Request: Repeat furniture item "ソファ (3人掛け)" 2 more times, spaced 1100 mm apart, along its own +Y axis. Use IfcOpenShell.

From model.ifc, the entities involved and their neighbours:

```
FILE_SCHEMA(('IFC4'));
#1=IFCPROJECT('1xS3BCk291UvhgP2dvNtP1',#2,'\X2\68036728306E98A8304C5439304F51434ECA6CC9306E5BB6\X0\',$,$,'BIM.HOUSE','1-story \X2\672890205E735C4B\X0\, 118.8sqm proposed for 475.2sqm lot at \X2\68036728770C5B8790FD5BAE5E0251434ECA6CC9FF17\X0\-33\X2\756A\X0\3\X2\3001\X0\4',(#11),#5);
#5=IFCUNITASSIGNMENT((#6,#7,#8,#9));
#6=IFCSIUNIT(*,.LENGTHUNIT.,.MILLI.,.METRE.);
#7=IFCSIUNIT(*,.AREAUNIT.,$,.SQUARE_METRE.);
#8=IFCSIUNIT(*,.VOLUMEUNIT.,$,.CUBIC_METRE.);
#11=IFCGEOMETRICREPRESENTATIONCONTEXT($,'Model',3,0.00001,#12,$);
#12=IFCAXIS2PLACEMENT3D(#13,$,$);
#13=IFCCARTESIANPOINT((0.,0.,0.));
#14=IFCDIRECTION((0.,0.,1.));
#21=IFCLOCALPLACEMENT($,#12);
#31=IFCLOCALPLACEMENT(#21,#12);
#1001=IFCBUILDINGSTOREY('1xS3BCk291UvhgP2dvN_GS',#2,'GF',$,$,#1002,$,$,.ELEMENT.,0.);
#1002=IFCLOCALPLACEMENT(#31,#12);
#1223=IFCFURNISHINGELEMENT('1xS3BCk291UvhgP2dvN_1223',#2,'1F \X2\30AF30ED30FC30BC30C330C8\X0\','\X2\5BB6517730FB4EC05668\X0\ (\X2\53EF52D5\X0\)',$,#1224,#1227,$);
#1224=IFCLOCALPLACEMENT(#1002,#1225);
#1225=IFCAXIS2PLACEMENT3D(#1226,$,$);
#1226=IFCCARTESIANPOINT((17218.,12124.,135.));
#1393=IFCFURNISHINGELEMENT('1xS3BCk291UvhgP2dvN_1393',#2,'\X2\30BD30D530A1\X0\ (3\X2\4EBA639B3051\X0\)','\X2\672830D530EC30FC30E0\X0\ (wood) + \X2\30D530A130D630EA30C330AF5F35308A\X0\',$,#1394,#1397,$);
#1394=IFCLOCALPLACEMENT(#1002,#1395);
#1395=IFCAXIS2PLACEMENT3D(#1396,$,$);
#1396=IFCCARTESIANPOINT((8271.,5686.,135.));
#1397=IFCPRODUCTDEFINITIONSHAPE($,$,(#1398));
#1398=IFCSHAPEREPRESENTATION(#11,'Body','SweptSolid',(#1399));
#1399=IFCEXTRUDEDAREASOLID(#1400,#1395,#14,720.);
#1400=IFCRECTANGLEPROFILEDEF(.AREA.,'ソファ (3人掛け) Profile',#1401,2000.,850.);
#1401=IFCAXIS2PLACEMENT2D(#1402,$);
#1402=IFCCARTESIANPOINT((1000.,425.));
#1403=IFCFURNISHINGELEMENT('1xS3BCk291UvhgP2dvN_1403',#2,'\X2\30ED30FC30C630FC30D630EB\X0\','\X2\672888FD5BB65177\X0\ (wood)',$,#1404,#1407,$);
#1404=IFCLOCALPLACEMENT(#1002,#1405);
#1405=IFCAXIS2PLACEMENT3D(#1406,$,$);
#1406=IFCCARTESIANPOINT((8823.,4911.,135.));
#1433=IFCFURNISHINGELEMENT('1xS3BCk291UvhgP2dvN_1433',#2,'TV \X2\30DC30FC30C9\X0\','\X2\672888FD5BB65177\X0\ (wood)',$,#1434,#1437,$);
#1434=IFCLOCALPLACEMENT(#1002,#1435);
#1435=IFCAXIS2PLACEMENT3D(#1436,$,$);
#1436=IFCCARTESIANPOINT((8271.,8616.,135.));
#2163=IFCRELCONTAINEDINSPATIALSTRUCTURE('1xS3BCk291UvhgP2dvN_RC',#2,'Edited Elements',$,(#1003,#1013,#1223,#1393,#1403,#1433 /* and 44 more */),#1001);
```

```python
import ifcopenshell
import ifcopenshell.api.geometry
import ifcopenshell.api.root
import ifcopenshell.util.element
import ifcopenshell.util.placement

model = ifcopenshell.open("model.ifc")


def reuse_history(source, copy):
    """copy_class also copies each property set's owner history, people and application; keep the originals."""
    for rel in copy.IsDefinedBy:
        if rel.is_a("IfcRelDefinesByProperties") and (history := rel.RelatingPropertyDefinition.OwnerHistory):
            rel.RelatingPropertyDefinition.OwnerHistory = source.OwnerHistory
            ifcopenshell.util.element.remove_deep2(model, history)


source = model.by_guid("1xS3BCk291UvhgP2dvN_1393")
base = ifcopenshell.util.placement.get_local_placement(source.ObjectPlacement)
step = base[:3, 1] * 1100.0

for i in range(1, 3):
    copy = ifcopenshell.api.root.copy_class(model, product=source)
    copy.Representation = ifcopenshell.util.element.copy_deep(
        model, source.Representation, exclude=["IfcGeometricRepresentationContext", "IfcRepresentationMap"]
    )
    reuse_history(source, copy)
    matrix = base.copy()
    matrix[:3, 3] += i * step
    print("added at", matrix[:3, 3].round(3) + 0.0)
    ifcopenshell.api.geometry.edit_object_placement(model, product=copy, matrix=matrix, is_si=False)

model.write("model_updated.ifc")
```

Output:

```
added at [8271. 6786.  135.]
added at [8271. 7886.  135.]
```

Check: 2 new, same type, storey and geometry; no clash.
